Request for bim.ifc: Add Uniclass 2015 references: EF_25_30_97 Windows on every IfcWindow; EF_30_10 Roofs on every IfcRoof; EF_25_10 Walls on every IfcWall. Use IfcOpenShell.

First a look at what the model holds.

```python
import ifcopenshell

model = ifcopenshell.open("bim.ifc")
print(model.schema)
print("classifications:", [c.Name for c in model.by_type("IfcClassification")])
for ifc_class in ("IfcDoor", "IfcRoof", "IfcStair", "IfcWall", "IfcWindow"):
    print(ifc_class, len(model.by_type(ifc_class)))
```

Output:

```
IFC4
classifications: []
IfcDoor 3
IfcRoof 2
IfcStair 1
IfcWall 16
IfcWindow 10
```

```python
import ifcopenshell
import ifcopenshell.api.classification

model = ifcopenshell.open("bim.ifc")

system = ifcopenshell.api.classification.add_classification(model, classification="Uniclass 2015")

codes = {
    "IfcWindow": ("EF_25_30_97", "Windows"),
    "IfcRoof": ("EF_30_10", "Roofs"),
    "IfcWall": ("EF_25_10", "Walls"),
}
for ifc_class, (code, name) in codes.items():
    products = model.by_type(ifc_class)
    ifcopenshell.api.classification.add_reference(
        model, products=products, classification=system, identification=code, name=name
    )
    print(code, len(products))

model.write("bim-out.ifc")
```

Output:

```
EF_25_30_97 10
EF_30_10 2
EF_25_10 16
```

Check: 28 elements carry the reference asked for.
